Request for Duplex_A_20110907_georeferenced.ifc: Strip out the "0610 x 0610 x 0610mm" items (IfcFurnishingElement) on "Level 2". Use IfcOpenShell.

First a look at what the model holds.

```python
import ifcopenshell
import ifcopenshell.util.element

model = ifcopenshell.open("Duplex_A_20110907_georeferenced.ifc")
print(model.schema)
storey = next(s for s in model.by_type("IfcBuildingStorey") if s.Name == "Level 2")
furniture = [e for e in ifcopenshell.util.element.get_decomposition(storey) if e.is_a("IfcFurnishingElement")]
seen = {}
for e in furniture:
    element_type = ifcopenshell.util.element.get_type(e)
    name = element_type.Name if element_type not in (None, e) else None
    seen[name] = seen.get(name, 0) + 1
for name, count in sorted(seen.items(), key=str):
    print(count, "x", name)
```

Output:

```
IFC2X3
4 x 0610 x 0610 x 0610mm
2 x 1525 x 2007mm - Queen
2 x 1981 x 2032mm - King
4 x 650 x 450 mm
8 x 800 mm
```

```python
import ifcopenshell
import ifcopenshell.api.root
import ifcopenshell.util.element

model = ifcopenshell.open("Duplex_A_20110907_georeferenced.ifc")

storey = next(s for s in model.by_type("IfcBuildingStorey") if s.Name == "Level 2")
furniture = [e for e in ifcopenshell.util.element.get_decomposition(storey) if e.is_a("IfcFurnishingElement")]
targets = [e for e in furniture if (t := ifcopenshell.util.element.get_type(e)) not in (None, e) and t.Name == "0610 x 0610 x 0610mm"]

for e in targets:
    ifcopenshell.api.root.remove_product(model, product=e)
print(len(targets), "removed")

model.write("Duplex_A_20110907_georeferenced-out.ifc")
```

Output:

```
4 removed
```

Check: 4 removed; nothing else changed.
